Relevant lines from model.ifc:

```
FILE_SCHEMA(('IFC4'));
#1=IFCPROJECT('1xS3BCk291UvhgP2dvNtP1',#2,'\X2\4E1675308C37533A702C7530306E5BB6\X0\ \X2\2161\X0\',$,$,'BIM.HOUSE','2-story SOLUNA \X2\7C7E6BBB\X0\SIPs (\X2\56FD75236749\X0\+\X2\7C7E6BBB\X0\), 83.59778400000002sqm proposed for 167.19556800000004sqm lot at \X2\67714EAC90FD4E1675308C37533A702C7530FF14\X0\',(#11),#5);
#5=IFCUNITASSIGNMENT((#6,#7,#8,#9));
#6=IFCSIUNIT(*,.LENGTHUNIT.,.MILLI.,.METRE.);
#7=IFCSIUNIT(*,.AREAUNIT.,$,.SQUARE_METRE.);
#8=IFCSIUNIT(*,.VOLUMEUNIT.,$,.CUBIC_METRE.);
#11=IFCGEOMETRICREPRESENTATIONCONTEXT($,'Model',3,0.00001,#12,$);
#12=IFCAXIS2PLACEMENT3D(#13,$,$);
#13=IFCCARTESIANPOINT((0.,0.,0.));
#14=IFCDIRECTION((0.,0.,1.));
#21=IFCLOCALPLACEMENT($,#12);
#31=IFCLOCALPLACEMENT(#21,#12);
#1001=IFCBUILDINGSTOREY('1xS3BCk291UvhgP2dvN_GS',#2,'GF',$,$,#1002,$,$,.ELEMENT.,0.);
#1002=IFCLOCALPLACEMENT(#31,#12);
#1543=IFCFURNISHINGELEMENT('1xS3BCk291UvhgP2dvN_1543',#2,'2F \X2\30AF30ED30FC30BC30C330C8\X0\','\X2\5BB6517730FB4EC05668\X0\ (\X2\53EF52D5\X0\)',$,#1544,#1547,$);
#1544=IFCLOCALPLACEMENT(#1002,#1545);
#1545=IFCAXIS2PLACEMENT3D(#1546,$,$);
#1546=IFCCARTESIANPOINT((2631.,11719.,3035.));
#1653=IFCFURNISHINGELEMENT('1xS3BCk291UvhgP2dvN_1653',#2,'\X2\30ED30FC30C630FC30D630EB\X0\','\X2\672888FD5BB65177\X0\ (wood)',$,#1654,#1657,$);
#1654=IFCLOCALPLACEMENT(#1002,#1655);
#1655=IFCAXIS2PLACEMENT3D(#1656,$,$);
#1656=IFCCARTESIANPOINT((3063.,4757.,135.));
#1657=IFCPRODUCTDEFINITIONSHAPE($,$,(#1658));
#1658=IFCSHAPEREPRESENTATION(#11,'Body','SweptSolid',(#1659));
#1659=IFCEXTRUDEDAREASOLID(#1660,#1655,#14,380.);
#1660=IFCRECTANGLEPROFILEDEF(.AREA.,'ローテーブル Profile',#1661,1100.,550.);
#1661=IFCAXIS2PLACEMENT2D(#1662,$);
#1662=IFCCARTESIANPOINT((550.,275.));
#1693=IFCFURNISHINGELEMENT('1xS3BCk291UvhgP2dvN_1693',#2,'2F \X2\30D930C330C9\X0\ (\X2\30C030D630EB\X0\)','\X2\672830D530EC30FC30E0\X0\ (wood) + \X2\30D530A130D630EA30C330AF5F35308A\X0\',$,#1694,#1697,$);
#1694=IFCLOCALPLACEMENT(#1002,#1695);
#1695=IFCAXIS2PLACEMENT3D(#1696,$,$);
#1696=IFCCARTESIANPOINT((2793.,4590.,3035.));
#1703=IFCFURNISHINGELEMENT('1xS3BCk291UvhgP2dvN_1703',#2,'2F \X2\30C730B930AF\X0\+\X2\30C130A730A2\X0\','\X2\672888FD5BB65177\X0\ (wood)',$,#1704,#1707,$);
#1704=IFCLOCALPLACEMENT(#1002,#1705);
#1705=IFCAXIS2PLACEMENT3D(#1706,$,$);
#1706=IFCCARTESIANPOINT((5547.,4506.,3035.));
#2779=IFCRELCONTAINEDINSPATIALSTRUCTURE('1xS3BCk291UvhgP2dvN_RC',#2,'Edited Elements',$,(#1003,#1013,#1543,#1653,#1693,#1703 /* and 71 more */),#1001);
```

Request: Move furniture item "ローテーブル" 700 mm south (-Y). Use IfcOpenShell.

```python
import ifcopenshell
import ifcopenshell.api.geometry
import ifcopenshell.util.placement
import ifcopenshell.util.unit

model = ifcopenshell.open("model.ifc")
unit_scale = ifcopenshell.util.unit.calculate_unit_scale(model)

item = model.by_guid("1xS3BCk291UvhgP2dvN_1653")
matrix = ifcopenshell.util.placement.get_local_placement(item.ObjectPlacement)
matrix[1, 3] -= 0.7 / unit_scale
ifcopenshell.api.geometry.edit_object_placement(model, product=item, matrix=matrix, is_si=False)

print(ifcopenshell.util.placement.get_local_placement(item.ObjectPlacement).round(3) + 0.0)

model.write("model_updated.ifc")
```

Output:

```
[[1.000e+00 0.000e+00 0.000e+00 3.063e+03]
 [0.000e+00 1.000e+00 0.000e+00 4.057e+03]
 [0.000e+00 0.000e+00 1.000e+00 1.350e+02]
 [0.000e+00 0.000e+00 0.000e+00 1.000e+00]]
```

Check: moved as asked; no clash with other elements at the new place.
